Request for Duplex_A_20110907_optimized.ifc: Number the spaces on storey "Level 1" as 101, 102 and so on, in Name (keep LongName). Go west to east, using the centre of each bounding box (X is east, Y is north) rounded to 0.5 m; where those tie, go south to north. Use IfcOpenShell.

First a look at what the model holds.

```python
import ifcopenshell
import ifcopenshell.util.element
import ifcopenshell.util.placement

model = ifcopenshell.open("Duplex_A_20110907_optimized.ifc")
print(model.schema)
storey = next(s for s in model.by_type("IfcBuildingStorey") if s.Name == "Level 1")
spaces = [e for e in ifcopenshell.util.element.get_decomposition(storey) if e.is_a("IfcSpace")]
for e in sorted(spaces, key=lambda e: e.id()):
    origin = ifcopenshell.util.placement.get_local_placement(e.ObjectPlacement)[:3, 3]
    print(e.id(), e.Name, e.LongName, origin.round(2) + 0.0, sep=" | ")
```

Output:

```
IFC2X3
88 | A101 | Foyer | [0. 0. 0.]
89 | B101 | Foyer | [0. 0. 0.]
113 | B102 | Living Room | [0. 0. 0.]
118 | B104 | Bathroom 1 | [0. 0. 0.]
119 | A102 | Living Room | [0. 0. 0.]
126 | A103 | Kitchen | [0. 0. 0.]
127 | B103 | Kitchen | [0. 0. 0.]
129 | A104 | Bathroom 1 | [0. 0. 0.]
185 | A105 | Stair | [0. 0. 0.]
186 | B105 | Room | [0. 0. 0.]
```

```python
import ifcopenshell
import ifcopenshell.geom
import ifcopenshell.util.element
import ifcopenshell.util.shape

model = ifcopenshell.open("Duplex_A_20110907_optimized.ifc")
settings = ifcopenshell.geom.settings()
settings.set("use-world-coords", True)


def centre(element):
    shape = ifcopenshell.geom.create_shape(settings, element)
    return ifcopenshell.util.shape.get_bbox_centroid(shape.geometry)


storey = next(s for s in model.by_type("IfcBuildingStorey") if s.Name == "Level 1")
spaces = [e for e in ifcopenshell.util.element.get_decomposition(storey) if e.is_a("IfcSpace")]

# Insertion points can sit at a corner or the storey origin, so sort by the geometry (in metres).
centres = {e: centre(e) for e in spaces}
spaces.sort(key=lambda e: (round(centres[e][0] / 0.5), centres[e][1]))

for i, e in enumerate(spaces, start=1):
    number = f"1{i:02d}"
    e.Name = number
    print(e.id(), number)

model.write("Duplex_A_20110907_optimized_rev.ifc")
```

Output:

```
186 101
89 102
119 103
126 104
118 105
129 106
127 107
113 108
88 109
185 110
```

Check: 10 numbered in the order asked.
